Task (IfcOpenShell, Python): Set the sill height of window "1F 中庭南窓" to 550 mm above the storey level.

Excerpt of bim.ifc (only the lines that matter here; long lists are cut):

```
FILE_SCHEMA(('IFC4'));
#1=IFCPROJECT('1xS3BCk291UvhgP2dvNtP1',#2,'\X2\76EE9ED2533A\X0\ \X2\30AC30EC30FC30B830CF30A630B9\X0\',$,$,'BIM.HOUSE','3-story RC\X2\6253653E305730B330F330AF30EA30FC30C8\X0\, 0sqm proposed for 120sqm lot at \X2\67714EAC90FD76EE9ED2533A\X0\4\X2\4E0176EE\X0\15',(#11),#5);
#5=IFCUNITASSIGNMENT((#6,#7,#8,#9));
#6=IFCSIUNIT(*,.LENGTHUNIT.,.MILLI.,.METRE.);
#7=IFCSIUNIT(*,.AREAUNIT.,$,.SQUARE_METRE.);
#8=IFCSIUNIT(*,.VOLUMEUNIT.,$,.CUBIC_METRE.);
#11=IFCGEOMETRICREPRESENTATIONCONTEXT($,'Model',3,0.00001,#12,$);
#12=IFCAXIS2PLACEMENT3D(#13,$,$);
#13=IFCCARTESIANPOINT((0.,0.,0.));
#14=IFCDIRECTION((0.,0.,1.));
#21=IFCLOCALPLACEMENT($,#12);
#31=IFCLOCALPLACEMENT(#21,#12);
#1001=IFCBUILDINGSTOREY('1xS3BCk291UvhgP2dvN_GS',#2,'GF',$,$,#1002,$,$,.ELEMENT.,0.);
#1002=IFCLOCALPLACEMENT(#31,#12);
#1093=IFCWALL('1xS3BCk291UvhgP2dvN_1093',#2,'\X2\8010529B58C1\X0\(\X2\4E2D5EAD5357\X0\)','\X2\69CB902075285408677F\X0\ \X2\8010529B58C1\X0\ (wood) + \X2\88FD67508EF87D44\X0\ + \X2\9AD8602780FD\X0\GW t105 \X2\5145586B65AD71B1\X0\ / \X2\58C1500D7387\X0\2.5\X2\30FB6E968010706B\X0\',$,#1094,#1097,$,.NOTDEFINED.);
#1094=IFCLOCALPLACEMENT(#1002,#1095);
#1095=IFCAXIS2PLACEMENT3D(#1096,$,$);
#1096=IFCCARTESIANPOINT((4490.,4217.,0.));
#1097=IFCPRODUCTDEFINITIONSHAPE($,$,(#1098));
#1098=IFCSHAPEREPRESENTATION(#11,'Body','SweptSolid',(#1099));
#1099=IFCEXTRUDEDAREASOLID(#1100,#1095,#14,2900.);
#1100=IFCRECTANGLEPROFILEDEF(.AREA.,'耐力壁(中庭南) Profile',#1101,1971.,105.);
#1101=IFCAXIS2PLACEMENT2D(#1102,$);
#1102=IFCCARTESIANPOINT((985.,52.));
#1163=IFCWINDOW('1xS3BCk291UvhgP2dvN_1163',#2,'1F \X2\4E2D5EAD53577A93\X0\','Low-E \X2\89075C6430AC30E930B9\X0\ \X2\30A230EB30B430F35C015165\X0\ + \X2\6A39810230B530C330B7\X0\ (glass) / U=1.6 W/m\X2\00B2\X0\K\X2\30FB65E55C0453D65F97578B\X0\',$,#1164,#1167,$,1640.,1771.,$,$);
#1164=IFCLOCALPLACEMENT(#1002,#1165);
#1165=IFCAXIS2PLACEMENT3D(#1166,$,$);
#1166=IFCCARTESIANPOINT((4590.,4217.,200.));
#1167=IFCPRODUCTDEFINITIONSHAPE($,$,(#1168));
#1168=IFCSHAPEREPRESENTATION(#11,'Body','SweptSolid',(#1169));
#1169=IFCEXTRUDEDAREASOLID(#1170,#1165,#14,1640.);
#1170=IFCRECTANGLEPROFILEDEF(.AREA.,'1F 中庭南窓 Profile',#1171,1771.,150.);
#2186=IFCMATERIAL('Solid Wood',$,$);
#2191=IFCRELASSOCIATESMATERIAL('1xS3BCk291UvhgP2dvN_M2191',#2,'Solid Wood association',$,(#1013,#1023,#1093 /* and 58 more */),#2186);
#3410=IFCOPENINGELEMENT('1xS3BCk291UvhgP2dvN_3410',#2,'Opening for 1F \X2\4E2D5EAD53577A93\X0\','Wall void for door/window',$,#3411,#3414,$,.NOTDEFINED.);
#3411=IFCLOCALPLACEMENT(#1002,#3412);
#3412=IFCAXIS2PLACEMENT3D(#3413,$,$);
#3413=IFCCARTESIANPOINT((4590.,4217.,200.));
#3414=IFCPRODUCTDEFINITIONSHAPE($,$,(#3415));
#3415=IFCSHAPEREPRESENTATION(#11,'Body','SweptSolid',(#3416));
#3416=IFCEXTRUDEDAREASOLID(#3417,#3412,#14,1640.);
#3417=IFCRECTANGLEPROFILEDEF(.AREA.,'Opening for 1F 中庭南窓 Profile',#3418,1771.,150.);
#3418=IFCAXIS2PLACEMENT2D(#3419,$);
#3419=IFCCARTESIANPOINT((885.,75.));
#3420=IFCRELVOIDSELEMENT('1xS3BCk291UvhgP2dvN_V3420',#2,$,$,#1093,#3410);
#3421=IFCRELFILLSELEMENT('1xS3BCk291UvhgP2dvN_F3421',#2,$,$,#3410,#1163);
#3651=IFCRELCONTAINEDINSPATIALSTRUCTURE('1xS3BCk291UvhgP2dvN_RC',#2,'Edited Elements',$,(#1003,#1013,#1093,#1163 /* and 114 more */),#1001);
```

```python
import numpy as np
import ifcopenshell
import ifcopenshell.api.geometry
import ifcopenshell.geom
import ifcopenshell.util.element
import ifcopenshell.util.placement
import ifcopenshell.util.shape
import ifcopenshell.util.unit

model = ifcopenshell.open("bim.ifc")
unit_scale = ifcopenshell.util.unit.calculate_unit_scale(model)

window = model.by_guid("1xS3BCk291UvhgP2dvN_1163")
opening = window.FillsVoids[0].RelatingOpeningElement
storey = ifcopenshell.util.element.get_container(window, ifc_class="IfcBuildingStorey")
level = ifcopenshell.util.placement.get_local_placement(storey.ObjectPlacement)[2, 3]

# The opening's origin need not be at the sill, so measure its lowest point.
shape = ifcopenshell.geom.create_shape(ifcopenshell.geom.settings(), opening)
bottom = ifcopenshell.util.shape.get_shape_bottom_elevation(shape, shape.geometry) / unit_scale
dz = level + 550.0 - bottom

shift = np.array([0.0, 0.0, dz])
# The window is not placed relative to its opening, so move both.
for product in (opening, window):
    matrix = ifcopenshell.util.placement.get_local_placement(product.ObjectPlacement)
    matrix[:3, 3] += shift
    ifcopenshell.api.geometry.edit_object_placement(model, product=product, matrix=matrix, is_si=False)

print(f"moved by {dz * unit_scale:+.3f} m")

model.write("bim_edited.ifc")
```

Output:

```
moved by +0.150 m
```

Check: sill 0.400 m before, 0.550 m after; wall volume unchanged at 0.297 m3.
